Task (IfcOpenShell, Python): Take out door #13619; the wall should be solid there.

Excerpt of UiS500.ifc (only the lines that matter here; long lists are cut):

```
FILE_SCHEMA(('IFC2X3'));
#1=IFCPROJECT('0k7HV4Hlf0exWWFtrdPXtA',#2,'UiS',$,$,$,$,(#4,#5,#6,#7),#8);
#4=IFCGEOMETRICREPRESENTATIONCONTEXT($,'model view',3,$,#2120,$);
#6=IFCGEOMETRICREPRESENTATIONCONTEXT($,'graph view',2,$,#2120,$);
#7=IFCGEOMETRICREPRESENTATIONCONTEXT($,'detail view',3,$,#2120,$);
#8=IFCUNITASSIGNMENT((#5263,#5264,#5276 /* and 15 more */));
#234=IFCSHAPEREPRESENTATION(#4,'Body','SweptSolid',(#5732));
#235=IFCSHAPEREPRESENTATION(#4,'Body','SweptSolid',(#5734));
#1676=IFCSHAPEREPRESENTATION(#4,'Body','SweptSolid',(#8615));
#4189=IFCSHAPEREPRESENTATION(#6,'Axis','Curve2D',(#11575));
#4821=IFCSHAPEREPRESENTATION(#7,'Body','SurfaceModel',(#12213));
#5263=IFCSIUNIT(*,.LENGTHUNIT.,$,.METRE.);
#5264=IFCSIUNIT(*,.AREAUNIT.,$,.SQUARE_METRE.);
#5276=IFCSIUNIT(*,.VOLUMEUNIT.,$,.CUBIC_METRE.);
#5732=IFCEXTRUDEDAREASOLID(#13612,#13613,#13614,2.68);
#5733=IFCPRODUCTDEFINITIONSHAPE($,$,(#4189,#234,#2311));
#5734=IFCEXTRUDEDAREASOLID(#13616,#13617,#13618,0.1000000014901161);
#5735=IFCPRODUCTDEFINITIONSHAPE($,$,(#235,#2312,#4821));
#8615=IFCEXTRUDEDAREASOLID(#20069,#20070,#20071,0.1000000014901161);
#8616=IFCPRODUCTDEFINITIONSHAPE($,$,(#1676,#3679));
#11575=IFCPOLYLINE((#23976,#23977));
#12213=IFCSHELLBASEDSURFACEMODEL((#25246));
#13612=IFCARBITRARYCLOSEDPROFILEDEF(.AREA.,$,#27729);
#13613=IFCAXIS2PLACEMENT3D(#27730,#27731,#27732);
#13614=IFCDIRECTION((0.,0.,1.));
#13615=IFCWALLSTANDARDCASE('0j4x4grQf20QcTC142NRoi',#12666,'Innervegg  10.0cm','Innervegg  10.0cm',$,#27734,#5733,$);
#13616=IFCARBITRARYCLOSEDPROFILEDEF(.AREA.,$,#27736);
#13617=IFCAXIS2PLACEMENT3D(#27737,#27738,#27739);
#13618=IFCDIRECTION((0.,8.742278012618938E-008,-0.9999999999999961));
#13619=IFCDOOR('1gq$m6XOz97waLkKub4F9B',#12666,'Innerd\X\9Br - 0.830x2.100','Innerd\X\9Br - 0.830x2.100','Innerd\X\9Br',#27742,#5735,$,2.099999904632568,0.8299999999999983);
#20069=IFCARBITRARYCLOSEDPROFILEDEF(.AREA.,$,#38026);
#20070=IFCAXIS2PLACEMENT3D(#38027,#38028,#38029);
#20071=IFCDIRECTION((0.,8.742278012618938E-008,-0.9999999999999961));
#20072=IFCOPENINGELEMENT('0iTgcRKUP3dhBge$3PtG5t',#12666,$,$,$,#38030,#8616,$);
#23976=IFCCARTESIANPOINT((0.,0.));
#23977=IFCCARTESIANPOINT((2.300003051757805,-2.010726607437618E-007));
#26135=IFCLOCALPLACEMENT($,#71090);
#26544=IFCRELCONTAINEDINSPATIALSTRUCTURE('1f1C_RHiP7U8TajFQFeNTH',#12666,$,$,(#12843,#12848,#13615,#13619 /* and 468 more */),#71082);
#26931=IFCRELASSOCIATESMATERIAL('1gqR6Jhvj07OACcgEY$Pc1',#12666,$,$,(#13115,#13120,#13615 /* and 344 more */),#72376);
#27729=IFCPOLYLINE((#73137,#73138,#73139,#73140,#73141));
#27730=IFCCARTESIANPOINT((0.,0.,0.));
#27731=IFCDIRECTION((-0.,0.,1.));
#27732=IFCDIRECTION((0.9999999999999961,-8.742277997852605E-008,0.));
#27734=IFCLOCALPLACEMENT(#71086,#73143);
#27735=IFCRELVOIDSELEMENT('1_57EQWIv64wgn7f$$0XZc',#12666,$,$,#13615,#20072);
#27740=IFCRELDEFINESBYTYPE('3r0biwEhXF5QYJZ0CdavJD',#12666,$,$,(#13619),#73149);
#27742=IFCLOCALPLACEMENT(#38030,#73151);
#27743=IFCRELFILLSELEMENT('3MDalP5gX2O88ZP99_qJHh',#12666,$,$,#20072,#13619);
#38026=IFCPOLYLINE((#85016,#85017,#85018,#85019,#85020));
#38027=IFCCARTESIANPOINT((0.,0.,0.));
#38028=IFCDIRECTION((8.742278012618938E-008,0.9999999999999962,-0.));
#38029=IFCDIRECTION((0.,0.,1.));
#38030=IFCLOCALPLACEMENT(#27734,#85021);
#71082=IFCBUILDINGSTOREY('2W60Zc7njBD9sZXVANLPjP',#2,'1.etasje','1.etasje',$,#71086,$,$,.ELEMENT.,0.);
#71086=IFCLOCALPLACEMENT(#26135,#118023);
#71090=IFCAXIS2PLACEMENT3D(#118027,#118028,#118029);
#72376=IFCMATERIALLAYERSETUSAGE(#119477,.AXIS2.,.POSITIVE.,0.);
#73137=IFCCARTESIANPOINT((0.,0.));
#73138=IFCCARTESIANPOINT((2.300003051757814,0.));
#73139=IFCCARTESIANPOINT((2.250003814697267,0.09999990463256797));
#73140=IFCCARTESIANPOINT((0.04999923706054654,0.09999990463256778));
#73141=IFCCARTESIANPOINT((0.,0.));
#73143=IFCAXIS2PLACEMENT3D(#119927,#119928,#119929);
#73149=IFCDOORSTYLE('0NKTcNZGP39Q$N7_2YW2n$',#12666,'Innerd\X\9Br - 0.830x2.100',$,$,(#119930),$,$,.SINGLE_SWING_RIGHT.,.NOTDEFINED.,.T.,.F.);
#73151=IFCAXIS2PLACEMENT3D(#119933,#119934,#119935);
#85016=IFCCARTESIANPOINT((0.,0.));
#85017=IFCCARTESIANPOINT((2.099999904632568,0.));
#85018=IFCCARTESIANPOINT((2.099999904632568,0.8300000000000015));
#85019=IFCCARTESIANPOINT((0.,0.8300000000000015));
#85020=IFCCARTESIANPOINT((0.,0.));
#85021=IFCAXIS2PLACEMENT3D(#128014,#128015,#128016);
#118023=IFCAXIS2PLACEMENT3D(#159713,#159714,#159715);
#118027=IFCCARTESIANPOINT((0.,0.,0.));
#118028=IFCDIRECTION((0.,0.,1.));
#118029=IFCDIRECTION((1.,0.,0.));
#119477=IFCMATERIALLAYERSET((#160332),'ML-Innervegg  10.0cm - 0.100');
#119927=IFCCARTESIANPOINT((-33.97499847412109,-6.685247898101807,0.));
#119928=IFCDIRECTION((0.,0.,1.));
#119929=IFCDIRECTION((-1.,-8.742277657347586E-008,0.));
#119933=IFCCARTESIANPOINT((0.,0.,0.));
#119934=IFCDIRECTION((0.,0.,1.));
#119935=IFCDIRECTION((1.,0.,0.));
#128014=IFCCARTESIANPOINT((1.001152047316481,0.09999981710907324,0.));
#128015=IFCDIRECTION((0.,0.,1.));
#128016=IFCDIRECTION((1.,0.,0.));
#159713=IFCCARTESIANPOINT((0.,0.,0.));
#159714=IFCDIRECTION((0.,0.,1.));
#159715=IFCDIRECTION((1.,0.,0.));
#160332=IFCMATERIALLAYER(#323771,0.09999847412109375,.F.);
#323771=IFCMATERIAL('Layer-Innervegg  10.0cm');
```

```python
import ifcopenshell
import ifcopenshell.api.feature
import ifcopenshell.api.root
import ifcopenshell.geom
import ifcopenshell.util.shape

model = ifcopenshell.open("UiS500.ifc")
settings = ifcopenshell.geom.settings()


def volume(element):
    """Net volume in cubic metres, openings subtracted."""
    shape = ifcopenshell.geom.create_shape(settings, element)
    return ifcopenshell.util.shape.get_volume(shape.geometry)


door = model.by_guid("1gq$m6XOz97waLkKub4F9B")
opening = door.FillsVoids[0].RelatingOpeningElement
wall = opening.VoidsElements[0].RelatingBuildingElement
before = volume(wall)

ifcopenshell.api.root.remove_product(model, product=door)
ifcopenshell.api.feature.remove_feature(model, feature=opening)

after = volume(wall)

print(f"wall volume {before:.3f} -> {after:.3f} m3")

model.write("UiS500-out.ifc")
```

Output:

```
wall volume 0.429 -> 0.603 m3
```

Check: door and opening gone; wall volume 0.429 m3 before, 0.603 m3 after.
